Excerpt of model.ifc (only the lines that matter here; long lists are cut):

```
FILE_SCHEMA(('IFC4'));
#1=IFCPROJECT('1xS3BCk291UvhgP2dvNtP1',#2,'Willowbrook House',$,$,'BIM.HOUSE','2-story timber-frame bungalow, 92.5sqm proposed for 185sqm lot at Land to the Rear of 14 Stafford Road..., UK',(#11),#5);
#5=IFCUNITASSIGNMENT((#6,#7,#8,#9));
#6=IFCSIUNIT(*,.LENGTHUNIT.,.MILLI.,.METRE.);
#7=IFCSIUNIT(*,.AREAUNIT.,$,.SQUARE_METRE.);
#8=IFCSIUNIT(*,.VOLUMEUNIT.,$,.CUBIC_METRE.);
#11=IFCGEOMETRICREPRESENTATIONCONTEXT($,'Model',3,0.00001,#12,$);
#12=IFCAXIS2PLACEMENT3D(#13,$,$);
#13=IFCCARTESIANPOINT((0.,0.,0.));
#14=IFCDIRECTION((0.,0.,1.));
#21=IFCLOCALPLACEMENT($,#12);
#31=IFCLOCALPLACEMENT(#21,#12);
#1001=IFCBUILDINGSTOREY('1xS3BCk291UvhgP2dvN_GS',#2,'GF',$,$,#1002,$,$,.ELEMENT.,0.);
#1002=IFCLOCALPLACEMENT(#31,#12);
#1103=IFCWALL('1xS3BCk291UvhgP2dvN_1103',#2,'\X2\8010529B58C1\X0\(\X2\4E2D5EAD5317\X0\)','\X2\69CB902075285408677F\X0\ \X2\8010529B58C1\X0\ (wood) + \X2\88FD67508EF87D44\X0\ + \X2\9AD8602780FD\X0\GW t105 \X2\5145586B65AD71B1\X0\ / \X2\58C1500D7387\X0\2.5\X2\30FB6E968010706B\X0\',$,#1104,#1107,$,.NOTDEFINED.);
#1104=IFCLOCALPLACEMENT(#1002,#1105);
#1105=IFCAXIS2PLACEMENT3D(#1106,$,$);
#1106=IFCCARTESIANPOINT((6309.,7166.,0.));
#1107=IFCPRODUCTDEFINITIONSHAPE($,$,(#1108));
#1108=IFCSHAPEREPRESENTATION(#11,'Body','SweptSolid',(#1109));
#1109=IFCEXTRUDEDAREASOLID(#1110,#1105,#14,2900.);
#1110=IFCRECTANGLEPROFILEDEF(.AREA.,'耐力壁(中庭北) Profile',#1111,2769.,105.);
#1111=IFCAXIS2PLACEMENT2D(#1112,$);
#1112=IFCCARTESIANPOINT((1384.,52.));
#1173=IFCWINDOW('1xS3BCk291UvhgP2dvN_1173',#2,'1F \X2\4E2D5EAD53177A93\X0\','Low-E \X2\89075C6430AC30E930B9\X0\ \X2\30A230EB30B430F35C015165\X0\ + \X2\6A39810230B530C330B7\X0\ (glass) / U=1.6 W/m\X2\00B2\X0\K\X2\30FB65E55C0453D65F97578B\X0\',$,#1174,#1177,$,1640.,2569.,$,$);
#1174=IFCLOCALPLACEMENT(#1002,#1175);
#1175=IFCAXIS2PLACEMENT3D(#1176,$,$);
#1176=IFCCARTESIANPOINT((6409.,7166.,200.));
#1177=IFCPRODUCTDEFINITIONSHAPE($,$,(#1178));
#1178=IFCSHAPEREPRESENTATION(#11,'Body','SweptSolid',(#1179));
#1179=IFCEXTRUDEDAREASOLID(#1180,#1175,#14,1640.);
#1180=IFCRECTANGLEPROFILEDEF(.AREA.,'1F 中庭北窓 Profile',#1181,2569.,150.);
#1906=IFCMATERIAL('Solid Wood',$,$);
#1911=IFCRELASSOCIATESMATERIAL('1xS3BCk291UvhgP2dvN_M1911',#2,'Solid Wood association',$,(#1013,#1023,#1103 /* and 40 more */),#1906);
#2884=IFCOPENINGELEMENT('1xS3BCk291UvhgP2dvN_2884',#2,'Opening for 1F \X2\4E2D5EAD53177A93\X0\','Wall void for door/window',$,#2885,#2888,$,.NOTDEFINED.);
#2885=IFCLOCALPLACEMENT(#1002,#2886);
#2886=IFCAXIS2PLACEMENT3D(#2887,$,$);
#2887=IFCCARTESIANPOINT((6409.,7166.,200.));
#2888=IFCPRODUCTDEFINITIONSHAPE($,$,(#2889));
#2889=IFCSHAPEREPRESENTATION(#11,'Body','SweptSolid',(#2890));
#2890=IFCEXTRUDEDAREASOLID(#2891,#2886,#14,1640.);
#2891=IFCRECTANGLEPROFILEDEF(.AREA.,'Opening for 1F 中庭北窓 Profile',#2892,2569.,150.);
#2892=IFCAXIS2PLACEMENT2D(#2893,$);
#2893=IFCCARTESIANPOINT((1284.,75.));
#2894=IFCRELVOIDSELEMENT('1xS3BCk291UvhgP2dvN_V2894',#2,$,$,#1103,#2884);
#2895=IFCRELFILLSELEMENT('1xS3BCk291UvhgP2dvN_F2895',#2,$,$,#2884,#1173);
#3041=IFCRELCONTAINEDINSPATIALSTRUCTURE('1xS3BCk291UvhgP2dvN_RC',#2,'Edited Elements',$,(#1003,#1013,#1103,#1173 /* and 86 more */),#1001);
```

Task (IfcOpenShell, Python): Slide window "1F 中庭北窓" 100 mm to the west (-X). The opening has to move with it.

```python
import ifcopenshell
import ifcopenshell.api.geometry
import ifcopenshell.util.placement
import ifcopenshell.util.unit

model = ifcopenshell.open("model.ifc")
unit_scale = ifcopenshell.util.unit.calculate_unit_scale(model)

window = model.by_guid("1xS3BCk291UvhgP2dvN_1173")
opening = window.FillsVoids[0].RelatingOpeningElement
wall = opening.VoidsElements[0].RelatingBuildingElement

wall_matrix = ifcopenshell.util.placement.get_local_placement(wall.ObjectPlacement)
shift = wall_matrix[:3, 0] * -0.1 / unit_scale
before = ifcopenshell.util.placement.get_local_placement(window.ObjectPlacement)[:3, 3].copy()

# The window is not placed relative to its opening, so move both.
for product in (opening, window):
    matrix = ifcopenshell.util.placement.get_local_placement(product.ObjectPlacement)
    matrix[:3, 3] += shift
    ifcopenshell.api.geometry.edit_object_placement(model, product=product, matrix=matrix, is_si=False)

after = ifcopenshell.util.placement.get_local_placement(window.ObjectPlacement)[:3, 3]
print("window moved by", (after - before).round(3) + 0.0)

model.write("model_rev.ifc")
```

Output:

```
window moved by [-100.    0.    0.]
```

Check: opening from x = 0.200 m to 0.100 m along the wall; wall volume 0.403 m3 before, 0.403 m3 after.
